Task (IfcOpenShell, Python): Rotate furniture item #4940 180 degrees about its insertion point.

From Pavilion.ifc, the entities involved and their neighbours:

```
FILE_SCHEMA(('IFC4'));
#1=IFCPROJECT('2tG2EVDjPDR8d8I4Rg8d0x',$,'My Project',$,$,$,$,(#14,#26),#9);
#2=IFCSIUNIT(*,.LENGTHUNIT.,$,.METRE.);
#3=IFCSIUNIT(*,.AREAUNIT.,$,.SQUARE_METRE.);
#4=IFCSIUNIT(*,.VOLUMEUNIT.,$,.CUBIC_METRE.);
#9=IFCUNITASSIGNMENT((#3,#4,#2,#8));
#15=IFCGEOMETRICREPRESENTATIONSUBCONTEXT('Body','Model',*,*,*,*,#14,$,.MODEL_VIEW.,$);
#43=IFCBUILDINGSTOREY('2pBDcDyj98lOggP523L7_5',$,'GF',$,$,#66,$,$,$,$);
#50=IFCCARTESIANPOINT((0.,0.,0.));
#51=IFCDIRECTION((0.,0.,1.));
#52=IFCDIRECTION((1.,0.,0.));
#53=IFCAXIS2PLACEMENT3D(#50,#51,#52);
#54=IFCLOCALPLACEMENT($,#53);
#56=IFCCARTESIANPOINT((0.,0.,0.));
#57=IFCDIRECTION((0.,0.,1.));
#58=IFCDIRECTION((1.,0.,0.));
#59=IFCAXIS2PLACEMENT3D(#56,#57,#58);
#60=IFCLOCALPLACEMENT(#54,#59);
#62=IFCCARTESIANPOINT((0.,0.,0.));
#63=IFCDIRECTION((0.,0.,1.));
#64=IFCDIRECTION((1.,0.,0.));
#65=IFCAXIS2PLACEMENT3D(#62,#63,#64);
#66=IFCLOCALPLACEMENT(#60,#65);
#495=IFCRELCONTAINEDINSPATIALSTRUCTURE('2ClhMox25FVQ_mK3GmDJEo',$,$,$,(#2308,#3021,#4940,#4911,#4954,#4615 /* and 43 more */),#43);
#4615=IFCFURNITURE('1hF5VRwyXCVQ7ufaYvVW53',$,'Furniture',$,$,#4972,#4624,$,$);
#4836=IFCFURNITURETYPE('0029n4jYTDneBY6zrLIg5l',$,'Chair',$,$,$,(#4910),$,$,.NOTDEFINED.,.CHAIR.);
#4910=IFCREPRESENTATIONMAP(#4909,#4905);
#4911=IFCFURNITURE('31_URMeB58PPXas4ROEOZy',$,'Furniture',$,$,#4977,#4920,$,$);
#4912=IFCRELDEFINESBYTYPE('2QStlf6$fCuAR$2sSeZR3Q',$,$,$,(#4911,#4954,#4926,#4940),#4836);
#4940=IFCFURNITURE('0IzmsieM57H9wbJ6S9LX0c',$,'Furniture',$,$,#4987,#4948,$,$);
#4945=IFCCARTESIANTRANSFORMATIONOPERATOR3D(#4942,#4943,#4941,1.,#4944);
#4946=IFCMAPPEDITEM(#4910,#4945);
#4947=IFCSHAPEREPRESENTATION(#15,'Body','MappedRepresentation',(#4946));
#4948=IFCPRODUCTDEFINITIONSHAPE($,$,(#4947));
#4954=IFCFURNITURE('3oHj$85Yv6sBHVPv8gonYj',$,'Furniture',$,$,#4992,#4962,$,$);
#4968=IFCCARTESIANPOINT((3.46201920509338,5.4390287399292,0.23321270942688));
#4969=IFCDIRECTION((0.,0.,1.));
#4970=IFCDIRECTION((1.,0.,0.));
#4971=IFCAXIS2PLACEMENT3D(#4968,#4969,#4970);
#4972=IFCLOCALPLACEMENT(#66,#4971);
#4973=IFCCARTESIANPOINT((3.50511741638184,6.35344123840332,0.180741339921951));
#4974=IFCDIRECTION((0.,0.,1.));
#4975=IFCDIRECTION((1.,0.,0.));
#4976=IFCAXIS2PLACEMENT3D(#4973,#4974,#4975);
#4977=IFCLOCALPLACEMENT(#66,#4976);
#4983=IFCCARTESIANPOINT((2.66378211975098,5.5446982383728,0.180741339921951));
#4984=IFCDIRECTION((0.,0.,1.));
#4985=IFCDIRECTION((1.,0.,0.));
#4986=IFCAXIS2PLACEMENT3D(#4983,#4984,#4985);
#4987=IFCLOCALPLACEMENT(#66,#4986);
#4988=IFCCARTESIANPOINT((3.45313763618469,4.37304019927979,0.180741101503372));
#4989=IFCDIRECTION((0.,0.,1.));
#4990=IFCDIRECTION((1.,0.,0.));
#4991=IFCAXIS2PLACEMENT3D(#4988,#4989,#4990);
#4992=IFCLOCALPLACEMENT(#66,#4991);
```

```python
import ifcopenshell
import ifcopenshell.api.geometry
import ifcopenshell.util.placement

model = ifcopenshell.open("Pavilion.ifc")

item = model.by_guid("0IzmsieM57H9wbJ6S9LX0c")
matrix = ifcopenshell.util.placement.get_local_placement(item.ObjectPlacement)
matrix = matrix @ ifcopenshell.util.placement.rotation(180, "Z")
ifcopenshell.api.geometry.edit_object_placement(model, product=item, matrix=matrix, is_si=False)

print(ifcopenshell.util.placement.get_local_placement(item.ObjectPlacement).round(3) + 0.0)

model.write("Pavilion-out.ifc")
```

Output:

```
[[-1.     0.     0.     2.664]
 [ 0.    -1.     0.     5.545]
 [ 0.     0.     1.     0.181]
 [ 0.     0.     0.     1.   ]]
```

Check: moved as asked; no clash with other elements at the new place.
